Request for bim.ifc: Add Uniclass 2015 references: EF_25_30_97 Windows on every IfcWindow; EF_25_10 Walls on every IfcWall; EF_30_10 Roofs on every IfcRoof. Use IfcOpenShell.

First a look at what the model holds.

```python
import ifcopenshell

model = ifcopenshell.open("bim.ifc")
print(model.schema)
print("classifications:", [c.Name for c in model.by_type("IfcClassification")])
for ifc_class in ("IfcDoor", "IfcRoof", "IfcStair", "IfcWall", "IfcWindow"):
    print(ifc_class, len(model.by_type(ifc_class)))
```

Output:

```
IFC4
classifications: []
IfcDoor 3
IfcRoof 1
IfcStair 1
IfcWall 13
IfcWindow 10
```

```python
import ifcopenshell
import ifcopenshell.api.classification

model = ifcopenshell.open("bim.ifc")

system = ifcopenshell.api.classification.add_classification(model, classification="Uniclass 2015")

codes = {
    "IfcWindow": ("EF_25_30_97", "Windows"),
    "IfcWall": ("EF_25_10", "Walls"),
    "IfcRoof": ("EF_30_10", "Roofs"),
}
for ifc_class, (code, name) in codes.items():
    products = model.by_type(ifc_class)
    ifcopenshell.api.classification.add_reference(
        model, products=products, classification=system, identification=code, name=name
    )
    print(code, len(products))

model.write("bim_v2.ifc")
```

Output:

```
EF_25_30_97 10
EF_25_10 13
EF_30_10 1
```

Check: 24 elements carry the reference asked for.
